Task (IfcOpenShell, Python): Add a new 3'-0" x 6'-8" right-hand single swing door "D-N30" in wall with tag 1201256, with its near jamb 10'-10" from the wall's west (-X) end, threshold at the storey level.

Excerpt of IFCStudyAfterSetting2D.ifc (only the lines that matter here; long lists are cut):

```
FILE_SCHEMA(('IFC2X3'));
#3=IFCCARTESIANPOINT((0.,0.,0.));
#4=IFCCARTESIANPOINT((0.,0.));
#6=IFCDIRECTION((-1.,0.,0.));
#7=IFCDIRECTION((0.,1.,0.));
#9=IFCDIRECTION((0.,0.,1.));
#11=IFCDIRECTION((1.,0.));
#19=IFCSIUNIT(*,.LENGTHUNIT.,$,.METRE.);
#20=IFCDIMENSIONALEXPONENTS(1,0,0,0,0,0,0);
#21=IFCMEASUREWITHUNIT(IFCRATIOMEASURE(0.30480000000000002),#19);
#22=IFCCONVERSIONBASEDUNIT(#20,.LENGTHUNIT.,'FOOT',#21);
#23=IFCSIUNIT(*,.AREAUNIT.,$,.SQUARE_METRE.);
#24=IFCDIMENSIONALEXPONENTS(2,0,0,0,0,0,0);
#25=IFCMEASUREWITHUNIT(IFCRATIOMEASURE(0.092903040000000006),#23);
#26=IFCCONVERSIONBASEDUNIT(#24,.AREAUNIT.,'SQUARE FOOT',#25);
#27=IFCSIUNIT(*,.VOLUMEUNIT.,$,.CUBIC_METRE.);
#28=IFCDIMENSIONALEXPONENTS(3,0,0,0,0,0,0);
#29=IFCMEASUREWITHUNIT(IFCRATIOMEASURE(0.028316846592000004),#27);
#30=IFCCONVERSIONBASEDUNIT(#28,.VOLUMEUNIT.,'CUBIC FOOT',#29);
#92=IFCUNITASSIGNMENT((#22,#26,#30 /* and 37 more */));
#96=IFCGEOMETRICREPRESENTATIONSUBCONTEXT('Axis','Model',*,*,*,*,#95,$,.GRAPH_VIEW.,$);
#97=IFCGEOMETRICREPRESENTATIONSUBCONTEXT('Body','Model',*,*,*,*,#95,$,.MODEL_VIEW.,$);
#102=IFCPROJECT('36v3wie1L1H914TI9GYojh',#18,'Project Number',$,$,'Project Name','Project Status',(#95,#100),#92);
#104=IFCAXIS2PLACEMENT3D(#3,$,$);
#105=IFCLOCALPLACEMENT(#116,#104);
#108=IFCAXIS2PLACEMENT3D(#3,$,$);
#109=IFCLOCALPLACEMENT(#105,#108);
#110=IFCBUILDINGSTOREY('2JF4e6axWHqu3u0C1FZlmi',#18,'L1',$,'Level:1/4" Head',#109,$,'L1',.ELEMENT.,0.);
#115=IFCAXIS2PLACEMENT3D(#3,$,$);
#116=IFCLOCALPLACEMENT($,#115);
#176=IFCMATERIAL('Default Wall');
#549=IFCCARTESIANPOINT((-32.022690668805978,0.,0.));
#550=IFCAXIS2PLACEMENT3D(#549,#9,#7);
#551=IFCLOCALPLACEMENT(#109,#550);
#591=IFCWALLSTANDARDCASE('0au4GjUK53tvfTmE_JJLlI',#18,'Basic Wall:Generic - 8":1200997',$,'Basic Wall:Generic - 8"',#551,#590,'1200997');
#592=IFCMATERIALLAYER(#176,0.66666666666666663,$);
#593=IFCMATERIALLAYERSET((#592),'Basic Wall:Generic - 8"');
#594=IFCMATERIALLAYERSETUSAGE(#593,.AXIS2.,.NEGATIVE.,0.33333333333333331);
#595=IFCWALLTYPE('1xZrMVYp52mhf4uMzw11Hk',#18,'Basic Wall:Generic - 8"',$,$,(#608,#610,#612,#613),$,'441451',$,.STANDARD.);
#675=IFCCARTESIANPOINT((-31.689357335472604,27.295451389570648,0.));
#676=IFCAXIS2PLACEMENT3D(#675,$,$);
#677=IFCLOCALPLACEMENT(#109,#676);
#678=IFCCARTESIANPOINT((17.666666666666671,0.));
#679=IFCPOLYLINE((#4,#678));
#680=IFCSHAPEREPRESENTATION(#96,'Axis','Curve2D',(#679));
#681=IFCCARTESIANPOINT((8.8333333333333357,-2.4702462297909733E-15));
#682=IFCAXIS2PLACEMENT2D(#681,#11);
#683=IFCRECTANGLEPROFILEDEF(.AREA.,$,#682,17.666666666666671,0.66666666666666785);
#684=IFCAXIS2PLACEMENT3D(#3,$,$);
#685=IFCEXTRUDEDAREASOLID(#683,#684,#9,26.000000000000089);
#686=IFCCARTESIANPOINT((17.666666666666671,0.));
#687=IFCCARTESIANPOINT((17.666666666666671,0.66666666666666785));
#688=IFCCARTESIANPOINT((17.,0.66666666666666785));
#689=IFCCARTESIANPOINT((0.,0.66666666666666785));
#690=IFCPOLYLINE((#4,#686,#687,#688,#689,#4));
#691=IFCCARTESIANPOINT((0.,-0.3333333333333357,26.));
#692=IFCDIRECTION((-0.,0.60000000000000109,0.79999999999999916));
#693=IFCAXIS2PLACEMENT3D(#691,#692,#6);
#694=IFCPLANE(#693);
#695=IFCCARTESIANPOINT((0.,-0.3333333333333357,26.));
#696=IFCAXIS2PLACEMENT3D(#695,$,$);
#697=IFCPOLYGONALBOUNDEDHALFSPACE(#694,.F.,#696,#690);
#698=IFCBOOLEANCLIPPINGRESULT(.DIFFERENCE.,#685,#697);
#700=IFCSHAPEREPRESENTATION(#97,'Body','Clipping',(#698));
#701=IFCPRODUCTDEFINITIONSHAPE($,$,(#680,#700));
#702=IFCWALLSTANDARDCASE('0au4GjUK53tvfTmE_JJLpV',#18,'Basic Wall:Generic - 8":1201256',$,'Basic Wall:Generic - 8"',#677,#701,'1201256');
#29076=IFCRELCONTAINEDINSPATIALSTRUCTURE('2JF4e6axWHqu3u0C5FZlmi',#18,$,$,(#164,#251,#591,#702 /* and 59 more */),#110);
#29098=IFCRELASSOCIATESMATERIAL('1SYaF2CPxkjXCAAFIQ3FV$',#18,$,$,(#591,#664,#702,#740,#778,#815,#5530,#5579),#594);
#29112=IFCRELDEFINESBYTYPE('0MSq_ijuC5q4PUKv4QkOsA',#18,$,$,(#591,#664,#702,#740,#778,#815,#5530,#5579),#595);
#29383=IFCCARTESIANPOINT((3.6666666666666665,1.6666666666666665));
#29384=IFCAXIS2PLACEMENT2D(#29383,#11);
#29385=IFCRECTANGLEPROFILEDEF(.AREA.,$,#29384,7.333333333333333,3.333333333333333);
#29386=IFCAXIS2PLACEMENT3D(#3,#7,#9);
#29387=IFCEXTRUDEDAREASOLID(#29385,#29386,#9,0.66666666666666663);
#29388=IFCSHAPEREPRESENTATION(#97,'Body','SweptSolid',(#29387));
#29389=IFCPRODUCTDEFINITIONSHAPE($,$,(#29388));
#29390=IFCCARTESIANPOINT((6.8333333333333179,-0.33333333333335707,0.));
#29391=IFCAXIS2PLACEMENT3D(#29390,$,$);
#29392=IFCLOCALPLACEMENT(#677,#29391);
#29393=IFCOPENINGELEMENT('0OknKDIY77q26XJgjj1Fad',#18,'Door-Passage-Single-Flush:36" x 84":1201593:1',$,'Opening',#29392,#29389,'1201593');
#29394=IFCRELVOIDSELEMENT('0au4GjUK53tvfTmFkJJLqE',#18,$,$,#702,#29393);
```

```python
import numpy as np
import ifcopenshell
import ifcopenshell.api.feature
import ifcopenshell.api.geometry
import ifcopenshell.api.root
import ifcopenshell.api.spatial
import ifcopenshell.api.type
import ifcopenshell.geom
import ifcopenshell.util.element
import ifcopenshell.util.placement
import ifcopenshell.util.representation
import ifcopenshell.util.shape
import ifcopenshell.util.unit

model = ifcopenshell.open("IFCStudyAfterSetting2D.ifc")
unit_scale = ifcopenshell.util.unit.calculate_unit_scale(model)
settings = ifcopenshell.geom.settings()


def volume(element):
    """Net volume in cubic metres, openings subtracted."""
    shape = ifcopenshell.geom.create_shape(settings, element)
    return ifcopenshell.util.shape.get_volume(shape.geometry)


wall = model.by_guid("0au4GjUK53tvfTmE_JJLpV")
storey = ifcopenshell.util.element.get_container(wall, ifc_class="IfcBuildingStorey")
context = ifcopenshell.util.representation.get_context(model, "Model", "Body", "MODEL_VIEW")
before = volume(wall)

width, height, from_end, sill = 0.9144, 2.032, 3.302, 0.0  # metres

# The wall runs along its own X axis, and the end named is its -X end.
wall_shape = ifcopenshell.geom.create_shape(settings, wall)
x, y, z = ifcopenshell.util.shape.get_vertices(wall_shape.geometry).T
start = x.min() + from_end
face, thickness = float(y.min()), float(y.max() - y.min())
wall_matrix = ifcopenshell.util.placement.get_local_placement(wall.ObjectPlacement)
level = ifcopenshell.util.placement.get_local_placement(storey.ObjectPlacement)[2, 3]


def in_wall(x, y):
    """Placement at x, y metres in the wall's axes, at sill height."""
    matrix = wall_matrix.copy()
    matrix[:, 3] = wall_matrix @ np.array([x / unit_scale, y / unit_scale, 0.0, 1.0])
    matrix[2, 3] = level + sill / unit_scale
    return matrix


# Opening: a box that overshoots both wall faces by 50 mm.
opening = ifcopenshell.api.root.create_entity(model, ifc_class="IfcOpeningElement")
box = ifcopenshell.api.geometry.add_wall_representation(
    model, context=context, length=width, height=height, thickness=thickness + 0.1
)
ifcopenshell.api.geometry.assign_representation(model, product=opening, representation=box)
ifcopenshell.api.geometry.edit_object_placement(model, product=opening, matrix=in_wall(start, face - 0.05), is_si=False)
ifcopenshell.api.feature.add_feature(model, feature=opening, element=wall)

door = ifcopenshell.api.root.create_entity(model, ifc_class="IfcDoor", name="D-N30")
door.OverallWidth, door.OverallHeight = width / unit_scale, height / unit_scale
body = ifcopenshell.api.geometry.add_door_representation(
    model,
    context=context,
    overall_width=door.OverallWidth,
    overall_height=door.OverallHeight,
    operation_type="SINGLE_SWING_RIGHT",
    lining_properties={"LiningDepth": thickness / unit_scale, "ThresholdDepth": thickness / unit_scale},
)
ifcopenshell.api.geometry.assign_representation(model, product=door, representation=body)
ifcopenshell.api.spatial.assign_container(model, products=[door], relating_structure=storey)
fills = ifcopenshell.api.feature.add_filling(model, opening=opening, element=door)
fills.OwnerHistory = door.OwnerHistory  # required in IFC2X3

# IFC2X3 keeps the operation on the door style.
style = ifcopenshell.api.root.create_entity(model, ifc_class="IfcDoorStyle", name="D-N30")
style.OperationType, style.ConstructionType = "SINGLE_SWING_RIGHT", "NOTDEFINED"
style.ParameterTakesPrecedence = style.Sizeable = False
ifcopenshell.api.type.assign_type(model, related_objects=[door], relating_type=style)

# The lining spans the wall, so the door starts at the wall face.
ifcopenshell.api.geometry.edit_object_placement(model, product=door, matrix=in_wall(start, face), is_si=False)

after = volume(wall)

print(f"wall volume {before:.3f} -> {after:.3f} m3")

model.write("IFCStudyAfterSetting2D_rev.ifc")
```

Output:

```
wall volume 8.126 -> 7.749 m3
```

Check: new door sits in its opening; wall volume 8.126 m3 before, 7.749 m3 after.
